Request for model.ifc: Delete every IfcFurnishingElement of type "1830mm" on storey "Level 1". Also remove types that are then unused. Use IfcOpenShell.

First a look at what the model holds.

```python
import ifcopenshell
import ifcopenshell.util.element

model = ifcopenshell.open("model.ifc")
print(model.schema)
storey = next(s for s in model.by_type("IfcBuildingStorey") if s.Name == "Level 1")
furniture = [e for e in ifcopenshell.util.element.get_decomposition(storey) if e.is_a("IfcFurnishingElement")]
seen = {}
for e in furniture:
    element_type = ifcopenshell.util.element.get_type(e)
    name = element_type.Name if element_type not in (None, e) else None
    seen[name] = seen.get(name, 0) + 1
for name, count in sorted(seen.items(), key=str):
    print(count, "x", name)
```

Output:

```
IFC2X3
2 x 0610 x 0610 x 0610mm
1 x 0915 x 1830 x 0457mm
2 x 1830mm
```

```python
import ifcopenshell
import ifcopenshell.api.root
import ifcopenshell.util.element

model = ifcopenshell.open("model.ifc")

storey = next(s for s in model.by_type("IfcBuildingStorey") if s.Name == "Level 1")
furniture = [e for e in ifcopenshell.util.element.get_decomposition(storey) if e.is_a("IfcFurnishingElement")]
targets = [e for e in furniture if (t := ifcopenshell.util.element.get_type(e)) not in (None, e) and t.Name == "1830mm"]
types = {ifcopenshell.util.element.get_type(e) for e in targets} - {None, *targets}

for e in targets:
    ifcopenshell.api.root.remove_product(model, product=e)
print(len(targets), "removed")

unused = [t for t in types if not ifcopenshell.util.element.get_types(t)]
for t in unused:
    ifcopenshell.api.root.remove_product(model, product=t)
print(len(unused), "unused types removed")

model.write("model_updated.ifc")
```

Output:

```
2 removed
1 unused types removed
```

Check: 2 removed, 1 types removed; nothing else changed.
